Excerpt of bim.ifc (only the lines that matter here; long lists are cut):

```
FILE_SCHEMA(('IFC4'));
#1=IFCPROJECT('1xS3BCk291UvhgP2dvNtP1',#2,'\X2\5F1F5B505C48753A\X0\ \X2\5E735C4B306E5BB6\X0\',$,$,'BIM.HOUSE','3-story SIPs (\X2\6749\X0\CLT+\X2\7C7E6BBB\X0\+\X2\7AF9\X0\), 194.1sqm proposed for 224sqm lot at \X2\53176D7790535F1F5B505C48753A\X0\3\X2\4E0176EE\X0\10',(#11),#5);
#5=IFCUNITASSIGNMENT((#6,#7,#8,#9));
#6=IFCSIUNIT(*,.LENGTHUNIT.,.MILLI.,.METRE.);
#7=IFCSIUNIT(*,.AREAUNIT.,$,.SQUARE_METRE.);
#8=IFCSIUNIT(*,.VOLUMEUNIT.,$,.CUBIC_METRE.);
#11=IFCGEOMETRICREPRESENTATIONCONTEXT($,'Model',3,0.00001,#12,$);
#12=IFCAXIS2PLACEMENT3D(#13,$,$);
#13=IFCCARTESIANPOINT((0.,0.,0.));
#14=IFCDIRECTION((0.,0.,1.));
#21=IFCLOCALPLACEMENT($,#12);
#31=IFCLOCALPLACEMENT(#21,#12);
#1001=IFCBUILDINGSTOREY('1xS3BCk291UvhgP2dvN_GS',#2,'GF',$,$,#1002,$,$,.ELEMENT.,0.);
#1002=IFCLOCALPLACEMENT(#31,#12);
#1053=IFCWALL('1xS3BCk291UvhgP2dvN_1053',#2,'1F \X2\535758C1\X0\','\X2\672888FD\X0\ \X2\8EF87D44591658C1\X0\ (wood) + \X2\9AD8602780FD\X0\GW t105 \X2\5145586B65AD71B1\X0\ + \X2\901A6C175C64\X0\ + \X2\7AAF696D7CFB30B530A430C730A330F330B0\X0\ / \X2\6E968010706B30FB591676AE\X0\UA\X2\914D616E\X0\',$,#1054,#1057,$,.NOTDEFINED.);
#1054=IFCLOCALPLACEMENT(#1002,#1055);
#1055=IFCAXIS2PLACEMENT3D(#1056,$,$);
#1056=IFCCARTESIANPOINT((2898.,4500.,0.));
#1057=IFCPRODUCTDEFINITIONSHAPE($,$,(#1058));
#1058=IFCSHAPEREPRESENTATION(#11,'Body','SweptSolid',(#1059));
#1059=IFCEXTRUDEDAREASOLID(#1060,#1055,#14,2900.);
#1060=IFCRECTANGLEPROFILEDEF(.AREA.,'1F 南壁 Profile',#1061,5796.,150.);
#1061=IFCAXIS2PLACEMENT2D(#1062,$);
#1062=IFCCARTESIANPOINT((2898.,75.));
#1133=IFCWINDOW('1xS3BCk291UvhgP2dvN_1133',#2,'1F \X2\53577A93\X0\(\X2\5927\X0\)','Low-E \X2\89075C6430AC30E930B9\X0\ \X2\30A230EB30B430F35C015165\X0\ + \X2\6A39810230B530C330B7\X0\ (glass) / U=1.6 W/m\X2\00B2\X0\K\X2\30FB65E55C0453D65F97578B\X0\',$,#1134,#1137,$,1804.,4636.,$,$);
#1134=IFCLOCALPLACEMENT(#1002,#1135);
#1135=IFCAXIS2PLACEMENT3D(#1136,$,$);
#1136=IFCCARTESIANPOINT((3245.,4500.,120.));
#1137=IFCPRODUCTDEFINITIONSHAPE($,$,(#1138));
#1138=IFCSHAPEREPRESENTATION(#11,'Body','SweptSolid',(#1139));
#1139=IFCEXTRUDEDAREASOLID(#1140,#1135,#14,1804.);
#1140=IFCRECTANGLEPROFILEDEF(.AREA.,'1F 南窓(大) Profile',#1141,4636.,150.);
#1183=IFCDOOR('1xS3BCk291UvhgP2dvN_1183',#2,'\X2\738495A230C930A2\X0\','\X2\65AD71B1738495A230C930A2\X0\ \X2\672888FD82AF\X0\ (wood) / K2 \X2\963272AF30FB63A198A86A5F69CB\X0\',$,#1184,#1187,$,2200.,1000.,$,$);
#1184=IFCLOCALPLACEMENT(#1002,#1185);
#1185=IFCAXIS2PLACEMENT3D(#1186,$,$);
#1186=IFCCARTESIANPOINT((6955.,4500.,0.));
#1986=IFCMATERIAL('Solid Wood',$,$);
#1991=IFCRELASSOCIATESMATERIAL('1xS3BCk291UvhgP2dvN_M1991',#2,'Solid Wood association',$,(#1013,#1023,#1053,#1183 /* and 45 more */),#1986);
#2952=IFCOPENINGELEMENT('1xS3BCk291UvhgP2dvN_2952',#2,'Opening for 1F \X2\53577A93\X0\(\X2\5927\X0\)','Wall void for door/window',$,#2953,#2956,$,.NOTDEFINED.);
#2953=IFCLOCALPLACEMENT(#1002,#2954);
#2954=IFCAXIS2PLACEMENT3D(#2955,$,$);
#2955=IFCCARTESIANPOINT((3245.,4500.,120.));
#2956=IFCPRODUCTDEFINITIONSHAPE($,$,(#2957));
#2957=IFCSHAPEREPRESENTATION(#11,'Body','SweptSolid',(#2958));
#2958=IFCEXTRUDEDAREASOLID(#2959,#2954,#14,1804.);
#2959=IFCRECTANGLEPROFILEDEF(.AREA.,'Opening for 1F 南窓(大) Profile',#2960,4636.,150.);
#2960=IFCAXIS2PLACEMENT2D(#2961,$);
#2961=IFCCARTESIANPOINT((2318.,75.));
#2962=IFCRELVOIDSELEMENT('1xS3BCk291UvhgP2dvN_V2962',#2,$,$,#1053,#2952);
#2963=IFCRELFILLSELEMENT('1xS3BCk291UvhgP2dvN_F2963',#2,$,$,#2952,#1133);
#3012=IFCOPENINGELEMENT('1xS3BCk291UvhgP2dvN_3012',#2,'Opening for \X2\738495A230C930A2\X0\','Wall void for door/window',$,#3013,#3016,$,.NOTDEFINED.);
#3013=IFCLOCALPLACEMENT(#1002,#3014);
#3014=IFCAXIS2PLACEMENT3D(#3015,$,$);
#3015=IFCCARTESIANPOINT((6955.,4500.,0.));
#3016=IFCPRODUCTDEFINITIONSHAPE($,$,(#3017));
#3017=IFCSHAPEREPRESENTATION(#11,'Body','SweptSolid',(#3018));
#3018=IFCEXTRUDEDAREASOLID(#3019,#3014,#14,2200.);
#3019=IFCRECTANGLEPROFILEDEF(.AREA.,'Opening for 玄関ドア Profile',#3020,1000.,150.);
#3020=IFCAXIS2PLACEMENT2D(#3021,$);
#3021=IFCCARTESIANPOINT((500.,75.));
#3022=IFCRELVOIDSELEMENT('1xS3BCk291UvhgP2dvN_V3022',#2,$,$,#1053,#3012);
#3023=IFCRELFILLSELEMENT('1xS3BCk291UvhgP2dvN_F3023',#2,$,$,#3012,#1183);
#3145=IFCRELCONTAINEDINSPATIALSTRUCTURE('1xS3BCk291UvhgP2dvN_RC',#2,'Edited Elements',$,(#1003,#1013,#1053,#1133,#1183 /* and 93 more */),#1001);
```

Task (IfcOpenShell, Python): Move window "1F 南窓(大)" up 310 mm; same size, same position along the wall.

```python
import numpy as np
import ifcopenshell
import ifcopenshell.api.geometry
import ifcopenshell.util.placement
import ifcopenshell.util.unit

model = ifcopenshell.open("bim.ifc")
unit_scale = ifcopenshell.util.unit.calculate_unit_scale(model)

window = model.by_guid("1xS3BCk291UvhgP2dvN_1133")
opening = window.FillsVoids[0].RelatingOpeningElement
dz = 0.31 / unit_scale

shift = np.array([0.0, 0.0, dz])
# The window is not placed relative to its opening, so move both.
for product in (opening, window):
    matrix = ifcopenshell.util.placement.get_local_placement(product.ObjectPlacement)
    matrix[:3, 3] += shift
    ifcopenshell.api.geometry.edit_object_placement(model, product=product, matrix=matrix, is_si=False)

print(f"moved by {dz * unit_scale:+.3f} m")

model.write("bim_rev.ifc")
```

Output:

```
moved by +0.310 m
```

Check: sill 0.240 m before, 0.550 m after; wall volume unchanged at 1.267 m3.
